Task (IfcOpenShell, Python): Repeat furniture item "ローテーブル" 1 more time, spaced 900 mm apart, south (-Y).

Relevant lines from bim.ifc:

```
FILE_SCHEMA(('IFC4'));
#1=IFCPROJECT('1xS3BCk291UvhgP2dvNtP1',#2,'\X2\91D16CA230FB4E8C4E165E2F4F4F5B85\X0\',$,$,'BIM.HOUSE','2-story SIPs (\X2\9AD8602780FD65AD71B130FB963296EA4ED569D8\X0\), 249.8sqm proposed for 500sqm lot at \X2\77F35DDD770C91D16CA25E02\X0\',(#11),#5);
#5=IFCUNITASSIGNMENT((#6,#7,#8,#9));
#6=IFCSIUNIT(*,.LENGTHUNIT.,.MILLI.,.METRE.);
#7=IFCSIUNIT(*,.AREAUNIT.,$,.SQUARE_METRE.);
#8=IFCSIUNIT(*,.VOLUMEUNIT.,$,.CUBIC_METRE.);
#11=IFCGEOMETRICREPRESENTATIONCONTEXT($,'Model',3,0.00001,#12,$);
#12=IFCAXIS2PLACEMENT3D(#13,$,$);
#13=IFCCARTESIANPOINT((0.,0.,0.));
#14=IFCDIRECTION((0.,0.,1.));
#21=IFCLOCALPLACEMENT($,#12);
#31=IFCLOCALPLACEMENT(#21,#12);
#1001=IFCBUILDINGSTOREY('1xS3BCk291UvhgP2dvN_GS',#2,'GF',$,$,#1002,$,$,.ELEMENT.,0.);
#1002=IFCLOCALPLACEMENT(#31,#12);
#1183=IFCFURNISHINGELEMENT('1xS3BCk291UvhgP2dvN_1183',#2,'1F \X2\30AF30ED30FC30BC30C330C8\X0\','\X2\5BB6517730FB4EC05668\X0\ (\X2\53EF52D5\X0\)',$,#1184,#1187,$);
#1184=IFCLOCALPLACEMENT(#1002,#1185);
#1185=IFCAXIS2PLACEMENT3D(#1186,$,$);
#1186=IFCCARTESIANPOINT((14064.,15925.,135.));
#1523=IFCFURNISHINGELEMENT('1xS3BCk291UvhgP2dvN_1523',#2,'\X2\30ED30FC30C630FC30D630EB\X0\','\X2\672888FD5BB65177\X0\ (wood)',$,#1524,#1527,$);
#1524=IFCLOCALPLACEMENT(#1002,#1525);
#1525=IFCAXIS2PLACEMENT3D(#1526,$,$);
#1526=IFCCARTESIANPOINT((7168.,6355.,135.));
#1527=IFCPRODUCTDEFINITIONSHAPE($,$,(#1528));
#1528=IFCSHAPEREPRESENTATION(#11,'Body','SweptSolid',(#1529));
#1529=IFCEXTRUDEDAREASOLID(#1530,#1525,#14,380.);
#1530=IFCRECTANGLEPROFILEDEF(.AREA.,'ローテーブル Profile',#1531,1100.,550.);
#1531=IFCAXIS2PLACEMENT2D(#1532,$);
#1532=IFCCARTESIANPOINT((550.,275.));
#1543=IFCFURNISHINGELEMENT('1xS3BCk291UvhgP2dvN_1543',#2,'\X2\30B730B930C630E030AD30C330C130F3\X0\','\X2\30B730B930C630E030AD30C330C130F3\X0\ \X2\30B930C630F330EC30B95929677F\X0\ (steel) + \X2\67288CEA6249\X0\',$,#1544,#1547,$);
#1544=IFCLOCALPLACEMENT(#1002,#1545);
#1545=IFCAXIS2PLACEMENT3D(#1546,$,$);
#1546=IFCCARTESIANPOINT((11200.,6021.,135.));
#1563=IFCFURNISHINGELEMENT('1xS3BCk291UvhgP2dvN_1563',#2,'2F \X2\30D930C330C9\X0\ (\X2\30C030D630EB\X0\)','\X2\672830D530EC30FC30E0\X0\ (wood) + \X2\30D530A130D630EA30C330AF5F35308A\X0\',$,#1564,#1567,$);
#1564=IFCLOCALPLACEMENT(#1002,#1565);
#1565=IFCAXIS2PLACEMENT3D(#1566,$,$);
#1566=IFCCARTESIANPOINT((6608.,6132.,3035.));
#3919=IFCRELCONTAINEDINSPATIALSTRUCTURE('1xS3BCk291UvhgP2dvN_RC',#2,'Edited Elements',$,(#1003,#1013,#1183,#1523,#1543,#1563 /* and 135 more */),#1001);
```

```python
import numpy as np
import ifcopenshell
import ifcopenshell.api.geometry
import ifcopenshell.api.root
import ifcopenshell.util.element
import ifcopenshell.util.placement

model = ifcopenshell.open("bim.ifc")


def reuse_history(source, copy):
    """copy_class also copies each property set's owner history, people and application; keep the originals."""
    for rel in copy.IsDefinedBy:
        if rel.is_a("IfcRelDefinesByProperties") and (history := rel.RelatingPropertyDefinition.OwnerHistory):
            rel.RelatingPropertyDefinition.OwnerHistory = source.OwnerHistory
            ifcopenshell.util.element.remove_deep2(model, history)


source = model.by_guid("1xS3BCk291UvhgP2dvN_1523")
base = ifcopenshell.util.placement.get_local_placement(source.ObjectPlacement)
step = np.array([0.0, -1.0, 0.0]) * 900.0

for i in range(1, 2):
    copy = ifcopenshell.api.root.copy_class(model, product=source)
    copy.Representation = ifcopenshell.util.element.copy_deep(
        model, source.Representation, exclude=["IfcGeometricRepresentationContext", "IfcRepresentationMap"]
    )
    reuse_history(source, copy)
    matrix = base.copy()
    matrix[:3, 3] += i * step
    print("added at", matrix[:3, 3].round(3) + 0.0)
    ifcopenshell.api.geometry.edit_object_placement(model, product=copy, matrix=matrix, is_si=False)

model.write("bim_edited.ifc")
```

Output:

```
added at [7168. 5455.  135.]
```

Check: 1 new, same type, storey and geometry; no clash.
